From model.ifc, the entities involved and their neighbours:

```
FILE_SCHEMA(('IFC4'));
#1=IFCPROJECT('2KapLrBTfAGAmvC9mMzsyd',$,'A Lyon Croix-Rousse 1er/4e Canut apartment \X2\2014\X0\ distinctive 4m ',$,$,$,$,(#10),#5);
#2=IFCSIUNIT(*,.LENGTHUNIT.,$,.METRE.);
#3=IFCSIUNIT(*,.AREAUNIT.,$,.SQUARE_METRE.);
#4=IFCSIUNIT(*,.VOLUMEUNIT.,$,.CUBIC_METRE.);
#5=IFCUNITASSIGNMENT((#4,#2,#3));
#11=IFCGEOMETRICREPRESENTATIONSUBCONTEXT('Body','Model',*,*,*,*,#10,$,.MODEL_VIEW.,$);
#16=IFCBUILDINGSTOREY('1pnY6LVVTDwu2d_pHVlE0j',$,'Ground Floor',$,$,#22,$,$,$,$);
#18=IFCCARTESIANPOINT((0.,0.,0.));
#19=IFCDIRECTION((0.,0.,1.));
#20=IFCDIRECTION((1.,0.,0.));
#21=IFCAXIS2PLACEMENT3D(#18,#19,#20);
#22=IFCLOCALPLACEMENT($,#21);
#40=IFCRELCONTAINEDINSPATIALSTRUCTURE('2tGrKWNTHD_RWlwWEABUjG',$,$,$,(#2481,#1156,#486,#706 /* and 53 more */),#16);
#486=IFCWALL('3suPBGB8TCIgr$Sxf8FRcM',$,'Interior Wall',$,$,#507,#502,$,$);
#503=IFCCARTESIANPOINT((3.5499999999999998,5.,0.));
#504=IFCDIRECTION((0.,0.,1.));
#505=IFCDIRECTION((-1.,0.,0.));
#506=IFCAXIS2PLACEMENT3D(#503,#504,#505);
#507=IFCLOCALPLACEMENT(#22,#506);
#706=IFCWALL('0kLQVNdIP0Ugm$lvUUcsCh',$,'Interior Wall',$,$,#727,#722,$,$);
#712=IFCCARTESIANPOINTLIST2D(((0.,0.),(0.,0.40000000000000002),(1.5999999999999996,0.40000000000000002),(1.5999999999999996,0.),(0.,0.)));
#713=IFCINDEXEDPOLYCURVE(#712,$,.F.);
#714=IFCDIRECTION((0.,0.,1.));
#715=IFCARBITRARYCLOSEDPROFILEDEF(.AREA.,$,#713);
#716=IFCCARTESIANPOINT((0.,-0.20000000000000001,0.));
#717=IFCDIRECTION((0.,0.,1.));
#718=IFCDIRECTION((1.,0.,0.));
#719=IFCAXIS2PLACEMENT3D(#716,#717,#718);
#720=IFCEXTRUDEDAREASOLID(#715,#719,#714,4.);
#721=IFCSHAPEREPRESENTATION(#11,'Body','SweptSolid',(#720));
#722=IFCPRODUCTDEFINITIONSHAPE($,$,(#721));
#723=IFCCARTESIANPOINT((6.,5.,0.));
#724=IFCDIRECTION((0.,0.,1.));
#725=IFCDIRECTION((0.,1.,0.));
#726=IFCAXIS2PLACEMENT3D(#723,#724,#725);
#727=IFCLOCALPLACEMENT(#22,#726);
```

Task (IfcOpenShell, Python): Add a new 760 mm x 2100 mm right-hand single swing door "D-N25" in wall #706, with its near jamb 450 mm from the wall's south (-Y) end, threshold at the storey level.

```python
import numpy as np
import ifcopenshell
import ifcopenshell.api.feature
import ifcopenshell.api.geometry
import ifcopenshell.api.root
import ifcopenshell.api.spatial
import ifcopenshell.geom
import ifcopenshell.util.element
import ifcopenshell.util.placement
import ifcopenshell.util.representation
import ifcopenshell.util.shape
import ifcopenshell.util.unit

model = ifcopenshell.open("model.ifc")
unit_scale = ifcopenshell.util.unit.calculate_unit_scale(model)
settings = ifcopenshell.geom.settings()


def volume(element):
    """Net volume in cubic metres, openings subtracted."""
    shape = ifcopenshell.geom.create_shape(settings, element)
    return ifcopenshell.util.shape.get_volume(shape.geometry)


wall = model.by_guid("0kLQVNdIP0Ugm$lvUUcsCh")
storey = ifcopenshell.util.element.get_container(wall, ifc_class="IfcBuildingStorey")
context = ifcopenshell.util.representation.get_context(model, "Model", "Body", "MODEL_VIEW")
before = volume(wall)

width, height, from_end, sill = 0.76, 2.1, 0.45, 0.0  # metres

# The wall runs along its own X axis, and the end named is its -X end.
wall_shape = ifcopenshell.geom.create_shape(settings, wall)
x, y, z = ifcopenshell.util.shape.get_vertices(wall_shape.geometry).T
start = x.min() + from_end
face, thickness = float(y.min()), float(y.max() - y.min())
wall_matrix = ifcopenshell.util.placement.get_local_placement(wall.ObjectPlacement)
level = ifcopenshell.util.placement.get_local_placement(storey.ObjectPlacement)[2, 3]


def in_wall(x, y):
    """Placement at x, y metres in the wall's axes, at sill height."""
    matrix = wall_matrix.copy()
    matrix[:, 3] = wall_matrix @ np.array([x / unit_scale, y / unit_scale, 0.0, 1.0])
    matrix[2, 3] = level + sill / unit_scale
    return matrix


# Opening: a box that overshoots both wall faces by 50 mm.
opening = ifcopenshell.api.root.create_entity(model, ifc_class="IfcOpeningElement", predefined_type="OPENING")
box = ifcopenshell.api.geometry.add_wall_representation(
    model, context=context, length=width, height=height, thickness=thickness + 0.1
)
ifcopenshell.api.geometry.assign_representation(model, product=opening, representation=box)
ifcopenshell.api.geometry.edit_object_placement(model, product=opening, matrix=in_wall(start, face - 0.05), is_si=False)
ifcopenshell.api.feature.add_feature(model, feature=opening, element=wall)

door = ifcopenshell.api.root.create_entity(model, ifc_class="IfcDoor", name="D-N25", predefined_type="DOOR")
door.OverallWidth, door.OverallHeight = width / unit_scale, height / unit_scale
door.OperationType = "SINGLE_SWING_RIGHT"
body = ifcopenshell.api.geometry.add_door_representation(
    model,
    context=context,
    overall_width=door.OverallWidth,
    overall_height=door.OverallHeight,
    operation_type="SINGLE_SWING_RIGHT",
    lining_properties={"LiningDepth": thickness / unit_scale, "ThresholdDepth": thickness / unit_scale},
)
ifcopenshell.api.geometry.assign_representation(model, product=door, representation=body)
ifcopenshell.api.spatial.assign_container(model, products=[door], relating_structure=storey)
ifcopenshell.api.feature.add_filling(model, opening=opening, element=door)

# The lining spans the wall, so the door starts at the wall face.
ifcopenshell.api.geometry.edit_object_placement(model, product=door, matrix=in_wall(start, face), is_si=False)

after = volume(wall)

print(f"wall volume {before:.3f} -> {after:.3f} m3")

model.write("model_edited.ifc")
```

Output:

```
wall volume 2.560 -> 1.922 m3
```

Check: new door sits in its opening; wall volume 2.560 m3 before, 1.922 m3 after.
